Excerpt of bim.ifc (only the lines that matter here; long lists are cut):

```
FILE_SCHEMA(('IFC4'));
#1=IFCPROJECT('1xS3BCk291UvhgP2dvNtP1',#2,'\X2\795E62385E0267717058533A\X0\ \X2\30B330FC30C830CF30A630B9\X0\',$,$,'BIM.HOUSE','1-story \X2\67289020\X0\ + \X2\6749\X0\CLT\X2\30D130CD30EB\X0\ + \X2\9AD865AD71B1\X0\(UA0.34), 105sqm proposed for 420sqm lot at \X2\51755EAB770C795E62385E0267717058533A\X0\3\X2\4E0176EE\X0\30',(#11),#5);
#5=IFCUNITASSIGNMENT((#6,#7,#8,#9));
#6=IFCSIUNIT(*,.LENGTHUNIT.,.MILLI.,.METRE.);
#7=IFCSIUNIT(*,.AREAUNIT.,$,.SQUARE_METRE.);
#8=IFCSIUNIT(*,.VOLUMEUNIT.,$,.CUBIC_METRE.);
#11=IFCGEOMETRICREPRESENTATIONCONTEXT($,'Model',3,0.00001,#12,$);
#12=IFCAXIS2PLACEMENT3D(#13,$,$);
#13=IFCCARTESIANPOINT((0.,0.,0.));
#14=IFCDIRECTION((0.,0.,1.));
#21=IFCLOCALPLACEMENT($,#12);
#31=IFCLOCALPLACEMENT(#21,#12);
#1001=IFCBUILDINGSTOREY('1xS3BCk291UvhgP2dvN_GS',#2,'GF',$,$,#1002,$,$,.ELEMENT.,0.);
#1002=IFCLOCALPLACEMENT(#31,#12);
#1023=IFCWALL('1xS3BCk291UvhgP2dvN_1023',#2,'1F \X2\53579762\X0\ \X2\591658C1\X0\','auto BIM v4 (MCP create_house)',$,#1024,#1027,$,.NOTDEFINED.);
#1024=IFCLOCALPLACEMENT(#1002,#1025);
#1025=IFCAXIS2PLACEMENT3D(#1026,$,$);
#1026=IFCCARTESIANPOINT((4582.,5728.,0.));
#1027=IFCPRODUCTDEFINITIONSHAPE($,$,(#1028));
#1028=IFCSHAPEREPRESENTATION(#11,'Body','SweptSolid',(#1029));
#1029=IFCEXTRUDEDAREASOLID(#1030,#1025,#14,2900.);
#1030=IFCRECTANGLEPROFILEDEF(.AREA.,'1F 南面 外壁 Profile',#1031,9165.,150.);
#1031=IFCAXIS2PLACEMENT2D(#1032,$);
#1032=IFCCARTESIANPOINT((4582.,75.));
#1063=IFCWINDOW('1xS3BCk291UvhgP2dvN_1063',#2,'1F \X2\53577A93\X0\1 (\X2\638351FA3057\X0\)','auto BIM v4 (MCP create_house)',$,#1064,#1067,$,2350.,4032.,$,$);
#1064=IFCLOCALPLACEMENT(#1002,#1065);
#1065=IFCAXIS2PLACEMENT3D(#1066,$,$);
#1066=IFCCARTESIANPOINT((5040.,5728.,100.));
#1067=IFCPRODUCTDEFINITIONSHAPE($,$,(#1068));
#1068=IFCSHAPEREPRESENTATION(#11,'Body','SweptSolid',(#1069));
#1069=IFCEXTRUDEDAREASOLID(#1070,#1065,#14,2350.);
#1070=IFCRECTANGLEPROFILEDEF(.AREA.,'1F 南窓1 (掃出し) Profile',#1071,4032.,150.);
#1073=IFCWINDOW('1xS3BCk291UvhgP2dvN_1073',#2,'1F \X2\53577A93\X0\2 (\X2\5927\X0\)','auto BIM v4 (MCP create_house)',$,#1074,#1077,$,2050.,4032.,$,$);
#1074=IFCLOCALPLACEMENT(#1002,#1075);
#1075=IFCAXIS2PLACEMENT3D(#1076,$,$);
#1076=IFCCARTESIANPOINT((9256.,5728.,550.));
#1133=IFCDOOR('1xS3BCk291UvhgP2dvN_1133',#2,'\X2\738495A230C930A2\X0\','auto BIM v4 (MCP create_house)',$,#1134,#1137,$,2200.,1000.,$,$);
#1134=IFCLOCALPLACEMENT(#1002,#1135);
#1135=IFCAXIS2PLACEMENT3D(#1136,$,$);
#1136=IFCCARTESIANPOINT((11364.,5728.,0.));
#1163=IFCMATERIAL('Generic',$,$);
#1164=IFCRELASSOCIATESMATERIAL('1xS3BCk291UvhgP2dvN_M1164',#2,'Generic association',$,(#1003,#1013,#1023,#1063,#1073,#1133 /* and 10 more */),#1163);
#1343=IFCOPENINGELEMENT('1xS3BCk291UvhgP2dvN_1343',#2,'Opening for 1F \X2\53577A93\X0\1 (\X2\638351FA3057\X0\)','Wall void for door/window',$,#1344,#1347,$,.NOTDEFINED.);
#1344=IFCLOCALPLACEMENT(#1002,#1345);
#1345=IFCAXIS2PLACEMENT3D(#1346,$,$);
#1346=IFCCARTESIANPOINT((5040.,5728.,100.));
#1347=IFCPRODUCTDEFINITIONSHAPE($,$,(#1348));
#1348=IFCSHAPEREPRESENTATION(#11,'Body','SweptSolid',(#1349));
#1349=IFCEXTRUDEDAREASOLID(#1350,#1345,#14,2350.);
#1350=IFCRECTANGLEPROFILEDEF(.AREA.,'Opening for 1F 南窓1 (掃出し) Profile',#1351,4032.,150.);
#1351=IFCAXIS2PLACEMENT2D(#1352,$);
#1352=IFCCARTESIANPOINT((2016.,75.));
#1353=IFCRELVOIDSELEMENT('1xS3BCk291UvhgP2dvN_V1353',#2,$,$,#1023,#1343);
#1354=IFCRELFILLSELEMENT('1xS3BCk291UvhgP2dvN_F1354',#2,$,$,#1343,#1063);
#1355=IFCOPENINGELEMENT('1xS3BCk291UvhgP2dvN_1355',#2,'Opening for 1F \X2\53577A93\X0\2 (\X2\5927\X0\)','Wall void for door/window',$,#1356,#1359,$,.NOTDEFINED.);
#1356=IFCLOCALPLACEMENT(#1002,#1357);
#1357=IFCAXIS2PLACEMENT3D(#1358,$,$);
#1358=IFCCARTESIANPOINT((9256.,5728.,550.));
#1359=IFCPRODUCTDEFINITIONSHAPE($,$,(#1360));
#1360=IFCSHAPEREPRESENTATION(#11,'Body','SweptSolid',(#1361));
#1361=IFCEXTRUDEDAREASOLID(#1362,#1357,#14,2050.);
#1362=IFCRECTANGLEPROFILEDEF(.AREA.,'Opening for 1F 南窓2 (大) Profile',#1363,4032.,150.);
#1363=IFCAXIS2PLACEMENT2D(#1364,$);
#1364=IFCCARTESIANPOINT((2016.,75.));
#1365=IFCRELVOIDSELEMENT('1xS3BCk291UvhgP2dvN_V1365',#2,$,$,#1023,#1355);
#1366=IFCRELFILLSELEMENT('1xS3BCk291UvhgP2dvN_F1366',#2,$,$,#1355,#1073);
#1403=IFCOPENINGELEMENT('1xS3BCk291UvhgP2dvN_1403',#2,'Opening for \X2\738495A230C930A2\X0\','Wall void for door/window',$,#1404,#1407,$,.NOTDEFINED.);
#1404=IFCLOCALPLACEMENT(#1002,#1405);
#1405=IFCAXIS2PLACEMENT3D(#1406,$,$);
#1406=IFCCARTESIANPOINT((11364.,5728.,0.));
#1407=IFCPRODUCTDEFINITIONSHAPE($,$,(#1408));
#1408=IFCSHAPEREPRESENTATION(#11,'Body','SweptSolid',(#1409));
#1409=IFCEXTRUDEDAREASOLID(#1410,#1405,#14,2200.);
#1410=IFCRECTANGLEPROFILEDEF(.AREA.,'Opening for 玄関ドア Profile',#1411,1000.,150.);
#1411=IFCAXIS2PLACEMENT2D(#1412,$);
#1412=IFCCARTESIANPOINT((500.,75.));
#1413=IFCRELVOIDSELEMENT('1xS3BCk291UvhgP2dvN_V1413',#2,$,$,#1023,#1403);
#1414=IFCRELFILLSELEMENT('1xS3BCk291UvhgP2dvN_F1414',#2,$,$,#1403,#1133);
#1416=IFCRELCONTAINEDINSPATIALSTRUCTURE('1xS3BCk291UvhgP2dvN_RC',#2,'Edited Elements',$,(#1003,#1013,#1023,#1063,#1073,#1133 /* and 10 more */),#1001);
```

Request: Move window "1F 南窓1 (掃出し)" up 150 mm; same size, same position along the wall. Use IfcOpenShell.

```python
import numpy as np
import ifcopenshell
import ifcopenshell.api.geometry
import ifcopenshell.util.placement
import ifcopenshell.util.unit

model = ifcopenshell.open("bim.ifc")
unit_scale = ifcopenshell.util.unit.calculate_unit_scale(model)

window = model.by_guid("1xS3BCk291UvhgP2dvN_1063")
opening = window.FillsVoids[0].RelatingOpeningElement
dz = 0.15 / unit_scale

shift = np.array([0.0, 0.0, dz])
# The window is not placed relative to its opening, so move both.
for product in (opening, window):
    matrix = ifcopenshell.util.placement.get_local_placement(product.ObjectPlacement)
    matrix[:3, 3] += shift
    ifcopenshell.api.geometry.edit_object_placement(model, product=product, matrix=matrix, is_si=False)

print(f"moved by {dz * unit_scale:+.3f} m")

model.write("bim_v2.ifc")
```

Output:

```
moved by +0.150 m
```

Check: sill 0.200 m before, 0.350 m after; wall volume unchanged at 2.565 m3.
